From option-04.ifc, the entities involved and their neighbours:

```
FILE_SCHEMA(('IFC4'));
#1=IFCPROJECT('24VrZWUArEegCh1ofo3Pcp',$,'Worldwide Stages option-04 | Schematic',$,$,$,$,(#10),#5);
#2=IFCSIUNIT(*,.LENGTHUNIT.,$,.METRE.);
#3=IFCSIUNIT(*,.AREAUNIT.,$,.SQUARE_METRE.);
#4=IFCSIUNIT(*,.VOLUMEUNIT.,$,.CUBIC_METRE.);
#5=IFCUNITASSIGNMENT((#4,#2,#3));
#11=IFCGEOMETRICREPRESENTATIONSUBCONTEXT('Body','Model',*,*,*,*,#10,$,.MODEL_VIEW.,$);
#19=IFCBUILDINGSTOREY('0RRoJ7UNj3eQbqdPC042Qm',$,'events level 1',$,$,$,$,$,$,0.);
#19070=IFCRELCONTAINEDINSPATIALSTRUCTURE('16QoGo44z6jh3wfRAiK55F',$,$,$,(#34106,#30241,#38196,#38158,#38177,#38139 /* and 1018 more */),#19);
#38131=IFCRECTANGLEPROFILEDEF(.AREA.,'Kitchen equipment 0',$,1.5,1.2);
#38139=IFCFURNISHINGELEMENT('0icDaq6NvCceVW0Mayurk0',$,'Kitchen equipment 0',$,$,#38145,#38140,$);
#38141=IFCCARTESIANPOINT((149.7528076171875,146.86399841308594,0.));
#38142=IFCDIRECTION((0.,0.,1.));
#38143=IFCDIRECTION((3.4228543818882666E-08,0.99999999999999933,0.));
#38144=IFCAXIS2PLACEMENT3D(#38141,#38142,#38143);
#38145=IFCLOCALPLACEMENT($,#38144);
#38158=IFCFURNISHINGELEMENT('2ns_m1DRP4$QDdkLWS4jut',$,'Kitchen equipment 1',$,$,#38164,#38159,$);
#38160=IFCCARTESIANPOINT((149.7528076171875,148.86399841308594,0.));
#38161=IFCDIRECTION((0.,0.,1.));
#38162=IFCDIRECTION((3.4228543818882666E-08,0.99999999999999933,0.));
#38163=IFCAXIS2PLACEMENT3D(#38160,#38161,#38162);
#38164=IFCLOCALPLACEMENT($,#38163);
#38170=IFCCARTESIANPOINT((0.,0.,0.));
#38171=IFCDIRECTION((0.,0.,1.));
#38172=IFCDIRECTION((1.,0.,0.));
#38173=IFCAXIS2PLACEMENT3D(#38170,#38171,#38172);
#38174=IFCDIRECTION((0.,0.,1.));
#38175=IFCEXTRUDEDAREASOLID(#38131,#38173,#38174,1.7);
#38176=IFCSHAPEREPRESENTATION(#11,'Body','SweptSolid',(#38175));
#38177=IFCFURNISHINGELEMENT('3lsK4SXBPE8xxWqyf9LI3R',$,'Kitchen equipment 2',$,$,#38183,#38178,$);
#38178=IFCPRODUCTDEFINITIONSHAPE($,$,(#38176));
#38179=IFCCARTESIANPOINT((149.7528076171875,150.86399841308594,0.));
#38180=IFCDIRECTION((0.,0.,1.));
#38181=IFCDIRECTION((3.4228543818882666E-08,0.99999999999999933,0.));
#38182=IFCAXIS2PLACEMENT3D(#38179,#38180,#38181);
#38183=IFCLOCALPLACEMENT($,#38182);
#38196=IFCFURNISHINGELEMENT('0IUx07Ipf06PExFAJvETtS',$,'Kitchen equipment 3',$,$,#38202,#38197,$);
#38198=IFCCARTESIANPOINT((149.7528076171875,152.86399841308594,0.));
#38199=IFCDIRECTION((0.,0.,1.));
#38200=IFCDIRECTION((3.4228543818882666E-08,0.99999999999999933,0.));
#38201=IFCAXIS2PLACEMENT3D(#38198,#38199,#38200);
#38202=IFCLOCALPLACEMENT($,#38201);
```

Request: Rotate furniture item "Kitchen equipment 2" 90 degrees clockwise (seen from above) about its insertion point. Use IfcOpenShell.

```python
import ifcopenshell
import ifcopenshell.api.geometry
import ifcopenshell.util.placement

model = ifcopenshell.open("option-04.ifc")

item = model.by_guid("3lsK4SXBPE8xxWqyf9LI3R")
matrix = ifcopenshell.util.placement.get_local_placement(item.ObjectPlacement)
matrix = matrix @ ifcopenshell.util.placement.rotation(-90, "Z")
ifcopenshell.api.geometry.edit_object_placement(model, product=item, matrix=matrix, is_si=False)

print(ifcopenshell.util.placement.get_local_placement(item.ObjectPlacement).round(3) + 0.0)

model.write("option-04_v2.ifc")
```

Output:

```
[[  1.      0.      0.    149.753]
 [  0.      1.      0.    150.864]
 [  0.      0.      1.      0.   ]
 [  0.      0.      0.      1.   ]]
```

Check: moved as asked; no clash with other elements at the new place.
